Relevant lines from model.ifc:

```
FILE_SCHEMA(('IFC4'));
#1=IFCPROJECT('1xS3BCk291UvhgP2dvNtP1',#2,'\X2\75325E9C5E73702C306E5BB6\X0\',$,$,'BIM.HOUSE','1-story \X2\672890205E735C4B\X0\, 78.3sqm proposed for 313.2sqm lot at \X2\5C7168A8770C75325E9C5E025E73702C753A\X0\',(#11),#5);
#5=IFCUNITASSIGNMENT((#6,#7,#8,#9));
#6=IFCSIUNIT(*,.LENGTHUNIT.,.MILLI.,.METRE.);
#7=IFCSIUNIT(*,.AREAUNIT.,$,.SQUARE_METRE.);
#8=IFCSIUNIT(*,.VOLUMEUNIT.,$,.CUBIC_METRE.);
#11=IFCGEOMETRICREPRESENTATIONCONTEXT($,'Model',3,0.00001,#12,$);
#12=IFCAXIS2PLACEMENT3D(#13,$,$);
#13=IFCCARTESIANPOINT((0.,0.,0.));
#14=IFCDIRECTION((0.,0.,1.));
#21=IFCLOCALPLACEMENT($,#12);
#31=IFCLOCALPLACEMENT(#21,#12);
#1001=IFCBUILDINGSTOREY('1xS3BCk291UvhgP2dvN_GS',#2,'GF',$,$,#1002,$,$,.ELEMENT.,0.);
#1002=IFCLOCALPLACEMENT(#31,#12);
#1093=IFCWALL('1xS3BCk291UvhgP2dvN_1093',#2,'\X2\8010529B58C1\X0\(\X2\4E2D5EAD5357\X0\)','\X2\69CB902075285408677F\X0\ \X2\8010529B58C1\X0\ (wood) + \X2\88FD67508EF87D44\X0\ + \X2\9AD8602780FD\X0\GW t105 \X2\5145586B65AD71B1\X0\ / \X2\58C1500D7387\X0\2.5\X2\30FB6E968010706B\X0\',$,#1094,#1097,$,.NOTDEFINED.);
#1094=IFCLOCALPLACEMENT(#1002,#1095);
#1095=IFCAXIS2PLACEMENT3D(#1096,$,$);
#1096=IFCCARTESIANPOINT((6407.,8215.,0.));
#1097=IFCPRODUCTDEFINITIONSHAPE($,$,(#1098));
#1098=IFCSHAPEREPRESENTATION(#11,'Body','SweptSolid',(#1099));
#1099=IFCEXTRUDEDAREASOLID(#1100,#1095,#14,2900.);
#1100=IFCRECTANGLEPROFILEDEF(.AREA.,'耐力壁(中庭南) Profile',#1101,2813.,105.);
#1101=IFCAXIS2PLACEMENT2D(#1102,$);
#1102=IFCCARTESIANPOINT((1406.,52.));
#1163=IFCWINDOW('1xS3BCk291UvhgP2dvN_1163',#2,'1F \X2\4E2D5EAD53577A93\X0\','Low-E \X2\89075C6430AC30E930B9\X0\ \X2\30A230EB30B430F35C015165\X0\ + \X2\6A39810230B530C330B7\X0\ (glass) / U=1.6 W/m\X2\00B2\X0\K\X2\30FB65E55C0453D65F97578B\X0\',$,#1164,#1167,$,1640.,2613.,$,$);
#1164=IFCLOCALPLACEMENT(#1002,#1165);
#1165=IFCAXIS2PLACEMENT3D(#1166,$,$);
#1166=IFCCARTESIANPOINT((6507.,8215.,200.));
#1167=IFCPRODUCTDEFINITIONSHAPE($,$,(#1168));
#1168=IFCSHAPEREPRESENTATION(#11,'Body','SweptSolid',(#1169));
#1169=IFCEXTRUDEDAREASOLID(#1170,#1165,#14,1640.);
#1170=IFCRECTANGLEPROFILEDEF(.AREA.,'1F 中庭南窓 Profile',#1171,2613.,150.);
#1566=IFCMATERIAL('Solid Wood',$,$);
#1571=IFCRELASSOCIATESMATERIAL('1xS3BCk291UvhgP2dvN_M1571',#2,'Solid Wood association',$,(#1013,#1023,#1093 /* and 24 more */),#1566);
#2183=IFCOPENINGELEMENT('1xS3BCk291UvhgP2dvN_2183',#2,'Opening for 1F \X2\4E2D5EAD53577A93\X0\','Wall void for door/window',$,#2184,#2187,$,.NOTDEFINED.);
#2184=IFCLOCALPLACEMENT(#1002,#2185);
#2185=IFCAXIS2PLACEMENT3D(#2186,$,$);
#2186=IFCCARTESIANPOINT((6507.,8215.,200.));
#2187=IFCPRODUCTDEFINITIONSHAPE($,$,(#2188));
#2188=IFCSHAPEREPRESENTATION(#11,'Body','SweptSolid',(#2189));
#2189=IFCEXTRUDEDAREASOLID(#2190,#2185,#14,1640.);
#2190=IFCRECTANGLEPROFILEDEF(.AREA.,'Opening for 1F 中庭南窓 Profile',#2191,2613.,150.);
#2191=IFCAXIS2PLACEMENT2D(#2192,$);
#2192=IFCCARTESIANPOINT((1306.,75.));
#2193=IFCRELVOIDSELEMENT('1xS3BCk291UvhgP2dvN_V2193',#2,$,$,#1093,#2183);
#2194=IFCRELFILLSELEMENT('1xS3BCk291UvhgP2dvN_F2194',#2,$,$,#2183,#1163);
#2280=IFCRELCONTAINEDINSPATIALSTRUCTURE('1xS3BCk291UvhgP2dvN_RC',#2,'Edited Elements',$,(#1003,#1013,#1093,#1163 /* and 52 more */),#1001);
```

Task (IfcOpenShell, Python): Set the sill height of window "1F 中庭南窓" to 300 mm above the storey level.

```python
import numpy as np
import ifcopenshell
import ifcopenshell.api.geometry
import ifcopenshell.geom
import ifcopenshell.util.element
import ifcopenshell.util.placement
import ifcopenshell.util.shape
import ifcopenshell.util.unit

model = ifcopenshell.open("model.ifc")
unit_scale = ifcopenshell.util.unit.calculate_unit_scale(model)

window = model.by_guid("1xS3BCk291UvhgP2dvN_1163")
opening = window.FillsVoids[0].RelatingOpeningElement
storey = ifcopenshell.util.element.get_container(window, ifc_class="IfcBuildingStorey")
level = ifcopenshell.util.placement.get_local_placement(storey.ObjectPlacement)[2, 3]

# The opening's origin need not be at the sill, so measure its lowest point.
shape = ifcopenshell.geom.create_shape(ifcopenshell.geom.settings(), opening)
bottom = ifcopenshell.util.shape.get_shape_bottom_elevation(shape, shape.geometry) / unit_scale
dz = level + 300.0 - bottom

shift = np.array([0.0, 0.0, dz])
# The window is not placed relative to its opening, so move both.
for product in (opening, window):
    matrix = ifcopenshell.util.placement.get_local_placement(product.ObjectPlacement)
    matrix[:3, 3] += shift
    ifcopenshell.api.geometry.edit_object_placement(model, product=product, matrix=matrix, is_si=False)

print(f"moved by {dz * unit_scale:+.3f} m")

model.write("model_updated.ifc")
```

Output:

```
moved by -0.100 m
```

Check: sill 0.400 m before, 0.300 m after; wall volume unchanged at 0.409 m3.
